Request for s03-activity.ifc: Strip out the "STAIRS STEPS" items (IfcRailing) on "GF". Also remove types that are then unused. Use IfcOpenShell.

First a look at what the model holds.

```python
import ifcopenshell
import ifcopenshell.util.element

model = ifcopenshell.open("s03-activity.ifc")
print(model.schema)
storey = next(s for s in model.by_type("IfcBuildingStorey") if s.Name == "GF")
railings = [e for e in ifcopenshell.util.element.get_decomposition(storey) if e.is_a("IfcRailing")]
seen = {}
for e in railings:
    element_type = ifcopenshell.util.element.get_type(e)
    name = element_type.Name if element_type not in (None, e) else None
    seen[name] = seen.get(name, 0) + 1
for name, count in sorted(seen.items(), key=str):
    print(count, "x", name)
```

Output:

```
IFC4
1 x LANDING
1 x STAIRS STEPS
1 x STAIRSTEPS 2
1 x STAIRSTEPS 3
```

```python
import ifcopenshell
import ifcopenshell.api.root
import ifcopenshell.util.element

model = ifcopenshell.open("s03-activity.ifc")

storey = next(s for s in model.by_type("IfcBuildingStorey") if s.Name == "GF")
railings = [e for e in ifcopenshell.util.element.get_decomposition(storey) if e.is_a("IfcRailing")]
targets = [e for e in railings if (t := ifcopenshell.util.element.get_type(e)) not in (None, e) and t.Name == "STAIRS STEPS"]
types = {ifcopenshell.util.element.get_type(e) for e in targets} - {None, *targets}

for e in targets:
    ifcopenshell.api.root.remove_product(model, product=e)
print(len(targets), "removed")

unused = [t for t in types if not ifcopenshell.util.element.get_types(t)]
for t in unused:
    ifcopenshell.api.root.remove_product(model, product=t)
print(len(unused), "unused types removed")

model.write("s03-activity_updated.ifc")
```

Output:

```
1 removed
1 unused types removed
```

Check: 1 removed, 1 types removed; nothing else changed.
